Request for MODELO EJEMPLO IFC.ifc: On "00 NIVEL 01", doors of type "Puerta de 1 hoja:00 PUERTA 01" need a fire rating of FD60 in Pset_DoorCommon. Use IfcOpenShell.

First a look at what the model holds.

```python
import ifcopenshell
import ifcopenshell.util.element

model = ifcopenshell.open("MODELO EJEMPLO IFC.ifc")
print(model.schema)
storey = next(s for s in model.by_type("IfcBuildingStorey") if s.Name == "00 NIVEL 01")
doors = [e for e in ifcopenshell.util.element.get_decomposition(storey) if e.is_a("IfcDoor")]
seen = {}
for e in doors:
    element_type = ifcopenshell.util.element.get_type(e)
    key = (element_type.Name if element_type != e and element_type else None, ifcopenshell.util.element.get_pset(e, "Pset_DoorCommon", "FireRating"))
    seen[key] = seen.get(key, 0) + 1
for (name, value), count in sorted(seen.items(), key=str):
    print(count, "x", name, "|", value)
```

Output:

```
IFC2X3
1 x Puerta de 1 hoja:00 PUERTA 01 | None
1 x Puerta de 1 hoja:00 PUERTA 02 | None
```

```python
import ifcopenshell
import ifcopenshell.api.pset
import ifcopenshell.util.element

model = ifcopenshell.open("MODELO EJEMPLO IFC.ifc")

storey = next(s for s in model.by_type("IfcBuildingStorey") if s.Name == "00 NIVEL 01")
doors = [e for e in ifcopenshell.util.element.get_decomposition(storey) if e.is_a("IfcDoor")]

count = 0
for e in doors:
    element_type = ifcopenshell.util.element.get_type(e)
    if element_type in (None, e) or element_type.Name != "Puerta de 1 hoja:00 PUERTA 01":
        continue
    # add_pset returns the element's existing set when there is one.
    pset = ifcopenshell.api.pset.add_pset(model, product=e, name="Pset_DoorCommon")
    ifcopenshell.api.pset.edit_pset(model, pset=pset, properties={"FireRating": "FD60"})
    count += 1

print(count, "doors updated")

model.write("MODELO EJEMPLO IFC_rev.ifc")
```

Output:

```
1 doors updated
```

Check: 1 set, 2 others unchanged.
